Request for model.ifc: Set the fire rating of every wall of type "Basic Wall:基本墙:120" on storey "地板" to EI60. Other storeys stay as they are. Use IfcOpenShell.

First a look at what the model holds.

```python
import ifcopenshell
import ifcopenshell.util.element

model = ifcopenshell.open("model.ifc")
print(model.schema)
storey = next(s for s in model.by_type("IfcBuildingStorey") if s.Name == "地板")
walls = [e for e in ifcopenshell.util.element.get_decomposition(storey) if e.is_a("IfcWall")]
seen = {}
for e in walls:
    element_type = ifcopenshell.util.element.get_type(e)
    key = (element_type.Name if element_type != e and element_type else None, ifcopenshell.util.element.get_pset(e, "Pset_WallCommon", "FireRating"))
    seen[key] = seen.get(key, 0) + 1
for (name, value), count in sorted(seen.items(), key=str):
    print(count, "x", name, "|", value)
```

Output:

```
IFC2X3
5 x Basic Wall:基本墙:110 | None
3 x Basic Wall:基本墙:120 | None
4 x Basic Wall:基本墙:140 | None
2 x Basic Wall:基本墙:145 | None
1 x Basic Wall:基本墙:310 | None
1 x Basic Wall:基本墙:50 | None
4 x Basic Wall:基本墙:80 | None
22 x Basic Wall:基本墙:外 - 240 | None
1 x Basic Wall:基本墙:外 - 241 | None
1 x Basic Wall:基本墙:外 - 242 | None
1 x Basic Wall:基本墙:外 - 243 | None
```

```python
import ifcopenshell
import ifcopenshell.api.pset
import ifcopenshell.util.element

model = ifcopenshell.open("model.ifc")

storey = next(s for s in model.by_type("IfcBuildingStorey") if s.Name == "地板")
walls = [e for e in ifcopenshell.util.element.get_decomposition(storey) if e.is_a("IfcWall")]

count = 0
for e in walls:
    element_type = ifcopenshell.util.element.get_type(e)
    if element_type in (None, e) or element_type.Name != "Basic Wall:基本墙:120":
        continue
    # add_pset returns the element's existing set when there is one.
    pset = ifcopenshell.api.pset.add_pset(model, product=e, name="Pset_WallCommon")
    ifcopenshell.api.pset.edit_pset(model, pset=pset, properties={"FireRating": "EI60"})
    count += 1

print(count, "walls updated")

model.write("model_v2.ifc")
```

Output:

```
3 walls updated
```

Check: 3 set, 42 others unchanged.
